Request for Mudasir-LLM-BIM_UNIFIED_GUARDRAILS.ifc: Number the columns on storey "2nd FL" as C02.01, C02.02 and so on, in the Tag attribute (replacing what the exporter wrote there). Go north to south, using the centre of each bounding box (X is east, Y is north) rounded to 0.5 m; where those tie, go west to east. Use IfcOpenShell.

First a look at what the model holds.

```python
import ifcopenshell
import ifcopenshell.util.element
import ifcopenshell.util.placement

model = ifcopenshell.open("Mudasir-LLM-BIM_UNIFIED_GUARDRAILS.ifc")
print(model.schema)
storey = next(s for s in model.by_type("IfcBuildingStorey") if s.Name == "2nd FL")
columns = [e for e in ifcopenshell.util.element.get_decomposition(storey) if e.is_a("IfcColumn")]
for e in sorted(columns, key=lambda e: e.id()):
    origin = ifcopenshell.util.placement.get_local_placement(e.ObjectPlacement)[:3, 3]
    print(e.id(), e.Tag, e.Name, origin.round(2) + 0.0, sep=" | ")
```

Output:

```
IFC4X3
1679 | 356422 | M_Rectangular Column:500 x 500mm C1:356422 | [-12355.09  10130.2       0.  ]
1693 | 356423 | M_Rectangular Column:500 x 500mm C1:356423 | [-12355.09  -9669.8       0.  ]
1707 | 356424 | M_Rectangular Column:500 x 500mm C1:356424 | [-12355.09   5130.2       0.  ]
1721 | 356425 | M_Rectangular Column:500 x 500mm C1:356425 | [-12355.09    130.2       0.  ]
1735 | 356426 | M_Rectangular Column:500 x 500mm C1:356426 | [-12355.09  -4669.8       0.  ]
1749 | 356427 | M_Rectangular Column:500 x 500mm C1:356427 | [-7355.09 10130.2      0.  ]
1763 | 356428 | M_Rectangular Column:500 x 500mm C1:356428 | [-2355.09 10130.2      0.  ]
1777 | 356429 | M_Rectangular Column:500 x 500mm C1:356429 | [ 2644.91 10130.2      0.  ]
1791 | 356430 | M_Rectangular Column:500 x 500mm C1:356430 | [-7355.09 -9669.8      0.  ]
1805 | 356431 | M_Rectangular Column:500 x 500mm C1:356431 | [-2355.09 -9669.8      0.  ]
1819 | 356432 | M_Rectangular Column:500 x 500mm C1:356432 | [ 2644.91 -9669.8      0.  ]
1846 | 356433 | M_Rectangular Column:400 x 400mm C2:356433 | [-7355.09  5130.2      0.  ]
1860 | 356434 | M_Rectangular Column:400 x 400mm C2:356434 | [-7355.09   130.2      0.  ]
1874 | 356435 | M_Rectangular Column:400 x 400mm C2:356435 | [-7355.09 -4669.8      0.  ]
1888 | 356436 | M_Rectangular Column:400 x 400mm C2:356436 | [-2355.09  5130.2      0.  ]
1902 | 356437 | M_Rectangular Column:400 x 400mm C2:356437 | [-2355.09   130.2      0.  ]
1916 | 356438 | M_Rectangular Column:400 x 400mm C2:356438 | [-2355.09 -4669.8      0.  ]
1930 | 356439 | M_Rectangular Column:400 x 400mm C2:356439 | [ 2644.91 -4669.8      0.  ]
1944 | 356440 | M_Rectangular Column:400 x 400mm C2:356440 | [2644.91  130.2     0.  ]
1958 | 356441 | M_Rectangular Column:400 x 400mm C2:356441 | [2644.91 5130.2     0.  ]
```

```python
import ifcopenshell
import ifcopenshell.geom
import ifcopenshell.util.element
import ifcopenshell.util.shape

model = ifcopenshell.open("Mudasir-LLM-BIM_UNIFIED_GUARDRAILS.ifc")
settings = ifcopenshell.geom.settings()
settings.set("use-world-coords", True)


def centre(element):
    shape = ifcopenshell.geom.create_shape(settings, element)
    return ifcopenshell.util.shape.get_bbox_centroid(shape.geometry)


storey = next(s for s in model.by_type("IfcBuildingStorey") if s.Name == "2nd FL")
columns = [e for e in ifcopenshell.util.element.get_decomposition(storey) if e.is_a("IfcColumn")]

# Insertion points can sit at a corner or the storey origin, so sort by the geometry (in metres).
centres = {e: centre(e) for e in columns}
columns.sort(key=lambda e: (-round(centres[e][1] / 0.5), centres[e][0]))

for i, e in enumerate(columns, start=1):
    number = f"C02.{i:02d}"
    e.Tag = number
    print(e.id(), number)

model.write("Mudasir-LLM-BIM_UNIFIED_GUARDRAILS-out.ifc")
```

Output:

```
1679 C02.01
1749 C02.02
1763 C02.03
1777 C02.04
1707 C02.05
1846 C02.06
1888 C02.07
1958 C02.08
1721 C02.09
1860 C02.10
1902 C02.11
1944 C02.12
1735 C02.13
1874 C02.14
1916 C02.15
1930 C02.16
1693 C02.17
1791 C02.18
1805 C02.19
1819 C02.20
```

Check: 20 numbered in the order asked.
